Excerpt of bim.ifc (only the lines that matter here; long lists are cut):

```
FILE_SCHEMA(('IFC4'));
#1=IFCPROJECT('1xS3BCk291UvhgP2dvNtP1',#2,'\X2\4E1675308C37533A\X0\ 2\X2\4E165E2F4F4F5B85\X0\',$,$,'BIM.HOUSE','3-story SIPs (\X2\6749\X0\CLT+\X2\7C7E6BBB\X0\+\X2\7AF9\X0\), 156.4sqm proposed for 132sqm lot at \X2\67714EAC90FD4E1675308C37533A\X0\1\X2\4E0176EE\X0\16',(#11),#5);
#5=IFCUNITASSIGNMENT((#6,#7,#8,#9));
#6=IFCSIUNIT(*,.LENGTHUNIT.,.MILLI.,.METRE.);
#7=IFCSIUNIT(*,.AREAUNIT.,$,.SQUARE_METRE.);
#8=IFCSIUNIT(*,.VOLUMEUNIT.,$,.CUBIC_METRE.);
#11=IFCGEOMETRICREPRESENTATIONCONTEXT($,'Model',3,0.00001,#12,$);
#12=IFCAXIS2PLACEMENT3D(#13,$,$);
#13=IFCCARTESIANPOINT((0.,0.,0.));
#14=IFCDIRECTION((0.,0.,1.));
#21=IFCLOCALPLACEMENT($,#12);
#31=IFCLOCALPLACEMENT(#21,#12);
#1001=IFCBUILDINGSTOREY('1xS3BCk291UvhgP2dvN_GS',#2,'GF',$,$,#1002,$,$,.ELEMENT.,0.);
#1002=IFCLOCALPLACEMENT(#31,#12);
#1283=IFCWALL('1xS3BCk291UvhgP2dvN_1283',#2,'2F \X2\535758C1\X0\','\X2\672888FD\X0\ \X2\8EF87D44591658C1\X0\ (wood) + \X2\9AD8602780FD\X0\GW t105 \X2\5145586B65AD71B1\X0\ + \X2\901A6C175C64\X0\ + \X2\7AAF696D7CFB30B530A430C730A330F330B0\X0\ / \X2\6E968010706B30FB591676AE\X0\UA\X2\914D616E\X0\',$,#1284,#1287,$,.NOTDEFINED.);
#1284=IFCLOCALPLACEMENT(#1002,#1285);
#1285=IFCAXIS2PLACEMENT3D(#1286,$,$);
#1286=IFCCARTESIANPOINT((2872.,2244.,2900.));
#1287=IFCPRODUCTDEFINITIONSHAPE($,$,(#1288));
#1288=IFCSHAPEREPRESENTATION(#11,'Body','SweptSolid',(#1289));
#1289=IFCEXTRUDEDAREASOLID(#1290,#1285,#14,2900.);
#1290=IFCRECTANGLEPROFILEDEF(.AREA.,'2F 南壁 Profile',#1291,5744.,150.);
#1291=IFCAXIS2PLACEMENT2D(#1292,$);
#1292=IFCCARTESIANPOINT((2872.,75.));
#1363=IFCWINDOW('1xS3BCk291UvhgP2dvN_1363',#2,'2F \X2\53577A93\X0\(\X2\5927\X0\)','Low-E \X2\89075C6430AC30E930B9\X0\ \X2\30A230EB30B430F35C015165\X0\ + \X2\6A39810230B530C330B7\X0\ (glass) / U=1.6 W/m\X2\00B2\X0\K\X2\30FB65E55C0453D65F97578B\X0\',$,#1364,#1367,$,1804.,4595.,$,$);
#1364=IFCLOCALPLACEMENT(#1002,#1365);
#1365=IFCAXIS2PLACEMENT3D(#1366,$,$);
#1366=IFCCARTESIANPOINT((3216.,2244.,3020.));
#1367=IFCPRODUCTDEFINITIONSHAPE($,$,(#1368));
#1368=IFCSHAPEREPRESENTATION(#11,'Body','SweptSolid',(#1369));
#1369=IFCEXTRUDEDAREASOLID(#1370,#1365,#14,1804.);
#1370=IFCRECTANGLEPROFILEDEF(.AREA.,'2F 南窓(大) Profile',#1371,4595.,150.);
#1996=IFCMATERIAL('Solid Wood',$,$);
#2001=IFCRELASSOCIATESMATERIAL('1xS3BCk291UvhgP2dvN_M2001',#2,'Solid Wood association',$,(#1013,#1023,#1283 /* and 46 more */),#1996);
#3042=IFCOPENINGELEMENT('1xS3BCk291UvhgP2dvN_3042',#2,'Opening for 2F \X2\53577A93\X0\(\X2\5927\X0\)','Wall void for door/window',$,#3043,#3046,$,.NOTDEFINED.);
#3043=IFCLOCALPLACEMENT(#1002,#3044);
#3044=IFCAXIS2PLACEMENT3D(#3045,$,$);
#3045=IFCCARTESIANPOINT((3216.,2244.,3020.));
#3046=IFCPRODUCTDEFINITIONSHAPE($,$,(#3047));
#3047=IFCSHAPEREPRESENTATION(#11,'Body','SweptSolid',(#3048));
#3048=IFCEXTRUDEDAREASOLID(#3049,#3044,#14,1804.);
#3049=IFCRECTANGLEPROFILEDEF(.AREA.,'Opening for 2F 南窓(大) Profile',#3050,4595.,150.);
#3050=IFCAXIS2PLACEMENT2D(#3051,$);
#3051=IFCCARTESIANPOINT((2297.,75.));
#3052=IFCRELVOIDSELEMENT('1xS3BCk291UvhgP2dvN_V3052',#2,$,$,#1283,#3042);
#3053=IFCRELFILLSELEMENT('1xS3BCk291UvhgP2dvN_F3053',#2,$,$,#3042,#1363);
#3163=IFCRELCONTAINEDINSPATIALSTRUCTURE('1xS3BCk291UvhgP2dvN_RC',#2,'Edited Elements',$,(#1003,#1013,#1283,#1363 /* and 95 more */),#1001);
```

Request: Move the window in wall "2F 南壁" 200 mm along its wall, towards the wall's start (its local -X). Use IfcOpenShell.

```python
import ifcopenshell
import ifcopenshell.api.geometry
import ifcopenshell.util.placement

model = ifcopenshell.open("bim.ifc")

window = model.by_id(1363)
opening = window.FillsVoids[0].RelatingOpeningElement
wall = opening.VoidsElements[0].RelatingBuildingElement

wall_matrix = ifcopenshell.util.placement.get_local_placement(wall.ObjectPlacement)
shift = wall_matrix[:3, 0] * -200.0
before = ifcopenshell.util.placement.get_local_placement(window.ObjectPlacement)[:3, 3].copy()

# The window is not placed relative to its opening, so move both.
for product in (opening, window):
    matrix = ifcopenshell.util.placement.get_local_placement(product.ObjectPlacement)
    matrix[:3, 3] += shift
    ifcopenshell.api.geometry.edit_object_placement(model, product=product, matrix=matrix, is_si=False)

after = ifcopenshell.util.placement.get_local_placement(window.ObjectPlacement)[:3, 3]
print("window moved by", (after - before).round(3) + 0.0)

model.write("bim_updated.ifc")
```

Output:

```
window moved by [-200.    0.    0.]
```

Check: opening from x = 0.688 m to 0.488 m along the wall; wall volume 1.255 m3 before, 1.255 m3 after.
